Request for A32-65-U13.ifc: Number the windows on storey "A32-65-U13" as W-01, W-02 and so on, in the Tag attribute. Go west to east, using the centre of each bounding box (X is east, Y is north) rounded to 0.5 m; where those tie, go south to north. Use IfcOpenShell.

First a look at what the model holds.

```python
import ifcopenshell
import ifcopenshell.util.element
import ifcopenshell.util.placement

model = ifcopenshell.open("A32-65-U13.ifc")
print(model.schema)
storey = next(s for s in model.by_type("IfcBuildingStorey") if s.Name == "A32-65-U13")
windows = [e for e in ifcopenshell.util.element.get_decomposition(storey) if e.is_a("IfcWindow")]
for e in sorted(windows, key=lambda e: e.id()):
    origin = ifcopenshell.util.placement.get_local_placement(e.ObjectPlacement)[:3, 3]
    print(e.id(), e.Tag, e.Name, origin.round(2) + 0.0, sep=" | ")
```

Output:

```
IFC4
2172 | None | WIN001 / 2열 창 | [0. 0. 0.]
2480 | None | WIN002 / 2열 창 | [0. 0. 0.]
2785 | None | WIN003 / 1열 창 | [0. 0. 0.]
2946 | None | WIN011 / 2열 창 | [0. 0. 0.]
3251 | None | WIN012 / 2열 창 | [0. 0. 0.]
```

```python
import ifcopenshell
import ifcopenshell.geom
import ifcopenshell.util.element
import ifcopenshell.util.shape

model = ifcopenshell.open("A32-65-U13.ifc")
settings = ifcopenshell.geom.settings()
settings.set("use-world-coords", True)


def centre(element):
    shape = ifcopenshell.geom.create_shape(settings, element)
    return ifcopenshell.util.shape.get_bbox_centroid(shape.geometry)


storey = next(s for s in model.by_type("IfcBuildingStorey") if s.Name == "A32-65-U13")
windows = [e for e in ifcopenshell.util.element.get_decomposition(storey) if e.is_a("IfcWindow")]

# Insertion points can sit at a corner or the storey origin, so sort by the geometry (in metres).
centres = {e: centre(e) for e in windows}
windows.sort(key=lambda e: (round(centres[e][0] / 0.5), centres[e][1]))

for i, e in enumerate(windows, start=1):
    number = f"W-{i:02d}"
    e.Tag = number
    print(e.id(), number)

model.write("A32-65-U13_v2.ifc")
```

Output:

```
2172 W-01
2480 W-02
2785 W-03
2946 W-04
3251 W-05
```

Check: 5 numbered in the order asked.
